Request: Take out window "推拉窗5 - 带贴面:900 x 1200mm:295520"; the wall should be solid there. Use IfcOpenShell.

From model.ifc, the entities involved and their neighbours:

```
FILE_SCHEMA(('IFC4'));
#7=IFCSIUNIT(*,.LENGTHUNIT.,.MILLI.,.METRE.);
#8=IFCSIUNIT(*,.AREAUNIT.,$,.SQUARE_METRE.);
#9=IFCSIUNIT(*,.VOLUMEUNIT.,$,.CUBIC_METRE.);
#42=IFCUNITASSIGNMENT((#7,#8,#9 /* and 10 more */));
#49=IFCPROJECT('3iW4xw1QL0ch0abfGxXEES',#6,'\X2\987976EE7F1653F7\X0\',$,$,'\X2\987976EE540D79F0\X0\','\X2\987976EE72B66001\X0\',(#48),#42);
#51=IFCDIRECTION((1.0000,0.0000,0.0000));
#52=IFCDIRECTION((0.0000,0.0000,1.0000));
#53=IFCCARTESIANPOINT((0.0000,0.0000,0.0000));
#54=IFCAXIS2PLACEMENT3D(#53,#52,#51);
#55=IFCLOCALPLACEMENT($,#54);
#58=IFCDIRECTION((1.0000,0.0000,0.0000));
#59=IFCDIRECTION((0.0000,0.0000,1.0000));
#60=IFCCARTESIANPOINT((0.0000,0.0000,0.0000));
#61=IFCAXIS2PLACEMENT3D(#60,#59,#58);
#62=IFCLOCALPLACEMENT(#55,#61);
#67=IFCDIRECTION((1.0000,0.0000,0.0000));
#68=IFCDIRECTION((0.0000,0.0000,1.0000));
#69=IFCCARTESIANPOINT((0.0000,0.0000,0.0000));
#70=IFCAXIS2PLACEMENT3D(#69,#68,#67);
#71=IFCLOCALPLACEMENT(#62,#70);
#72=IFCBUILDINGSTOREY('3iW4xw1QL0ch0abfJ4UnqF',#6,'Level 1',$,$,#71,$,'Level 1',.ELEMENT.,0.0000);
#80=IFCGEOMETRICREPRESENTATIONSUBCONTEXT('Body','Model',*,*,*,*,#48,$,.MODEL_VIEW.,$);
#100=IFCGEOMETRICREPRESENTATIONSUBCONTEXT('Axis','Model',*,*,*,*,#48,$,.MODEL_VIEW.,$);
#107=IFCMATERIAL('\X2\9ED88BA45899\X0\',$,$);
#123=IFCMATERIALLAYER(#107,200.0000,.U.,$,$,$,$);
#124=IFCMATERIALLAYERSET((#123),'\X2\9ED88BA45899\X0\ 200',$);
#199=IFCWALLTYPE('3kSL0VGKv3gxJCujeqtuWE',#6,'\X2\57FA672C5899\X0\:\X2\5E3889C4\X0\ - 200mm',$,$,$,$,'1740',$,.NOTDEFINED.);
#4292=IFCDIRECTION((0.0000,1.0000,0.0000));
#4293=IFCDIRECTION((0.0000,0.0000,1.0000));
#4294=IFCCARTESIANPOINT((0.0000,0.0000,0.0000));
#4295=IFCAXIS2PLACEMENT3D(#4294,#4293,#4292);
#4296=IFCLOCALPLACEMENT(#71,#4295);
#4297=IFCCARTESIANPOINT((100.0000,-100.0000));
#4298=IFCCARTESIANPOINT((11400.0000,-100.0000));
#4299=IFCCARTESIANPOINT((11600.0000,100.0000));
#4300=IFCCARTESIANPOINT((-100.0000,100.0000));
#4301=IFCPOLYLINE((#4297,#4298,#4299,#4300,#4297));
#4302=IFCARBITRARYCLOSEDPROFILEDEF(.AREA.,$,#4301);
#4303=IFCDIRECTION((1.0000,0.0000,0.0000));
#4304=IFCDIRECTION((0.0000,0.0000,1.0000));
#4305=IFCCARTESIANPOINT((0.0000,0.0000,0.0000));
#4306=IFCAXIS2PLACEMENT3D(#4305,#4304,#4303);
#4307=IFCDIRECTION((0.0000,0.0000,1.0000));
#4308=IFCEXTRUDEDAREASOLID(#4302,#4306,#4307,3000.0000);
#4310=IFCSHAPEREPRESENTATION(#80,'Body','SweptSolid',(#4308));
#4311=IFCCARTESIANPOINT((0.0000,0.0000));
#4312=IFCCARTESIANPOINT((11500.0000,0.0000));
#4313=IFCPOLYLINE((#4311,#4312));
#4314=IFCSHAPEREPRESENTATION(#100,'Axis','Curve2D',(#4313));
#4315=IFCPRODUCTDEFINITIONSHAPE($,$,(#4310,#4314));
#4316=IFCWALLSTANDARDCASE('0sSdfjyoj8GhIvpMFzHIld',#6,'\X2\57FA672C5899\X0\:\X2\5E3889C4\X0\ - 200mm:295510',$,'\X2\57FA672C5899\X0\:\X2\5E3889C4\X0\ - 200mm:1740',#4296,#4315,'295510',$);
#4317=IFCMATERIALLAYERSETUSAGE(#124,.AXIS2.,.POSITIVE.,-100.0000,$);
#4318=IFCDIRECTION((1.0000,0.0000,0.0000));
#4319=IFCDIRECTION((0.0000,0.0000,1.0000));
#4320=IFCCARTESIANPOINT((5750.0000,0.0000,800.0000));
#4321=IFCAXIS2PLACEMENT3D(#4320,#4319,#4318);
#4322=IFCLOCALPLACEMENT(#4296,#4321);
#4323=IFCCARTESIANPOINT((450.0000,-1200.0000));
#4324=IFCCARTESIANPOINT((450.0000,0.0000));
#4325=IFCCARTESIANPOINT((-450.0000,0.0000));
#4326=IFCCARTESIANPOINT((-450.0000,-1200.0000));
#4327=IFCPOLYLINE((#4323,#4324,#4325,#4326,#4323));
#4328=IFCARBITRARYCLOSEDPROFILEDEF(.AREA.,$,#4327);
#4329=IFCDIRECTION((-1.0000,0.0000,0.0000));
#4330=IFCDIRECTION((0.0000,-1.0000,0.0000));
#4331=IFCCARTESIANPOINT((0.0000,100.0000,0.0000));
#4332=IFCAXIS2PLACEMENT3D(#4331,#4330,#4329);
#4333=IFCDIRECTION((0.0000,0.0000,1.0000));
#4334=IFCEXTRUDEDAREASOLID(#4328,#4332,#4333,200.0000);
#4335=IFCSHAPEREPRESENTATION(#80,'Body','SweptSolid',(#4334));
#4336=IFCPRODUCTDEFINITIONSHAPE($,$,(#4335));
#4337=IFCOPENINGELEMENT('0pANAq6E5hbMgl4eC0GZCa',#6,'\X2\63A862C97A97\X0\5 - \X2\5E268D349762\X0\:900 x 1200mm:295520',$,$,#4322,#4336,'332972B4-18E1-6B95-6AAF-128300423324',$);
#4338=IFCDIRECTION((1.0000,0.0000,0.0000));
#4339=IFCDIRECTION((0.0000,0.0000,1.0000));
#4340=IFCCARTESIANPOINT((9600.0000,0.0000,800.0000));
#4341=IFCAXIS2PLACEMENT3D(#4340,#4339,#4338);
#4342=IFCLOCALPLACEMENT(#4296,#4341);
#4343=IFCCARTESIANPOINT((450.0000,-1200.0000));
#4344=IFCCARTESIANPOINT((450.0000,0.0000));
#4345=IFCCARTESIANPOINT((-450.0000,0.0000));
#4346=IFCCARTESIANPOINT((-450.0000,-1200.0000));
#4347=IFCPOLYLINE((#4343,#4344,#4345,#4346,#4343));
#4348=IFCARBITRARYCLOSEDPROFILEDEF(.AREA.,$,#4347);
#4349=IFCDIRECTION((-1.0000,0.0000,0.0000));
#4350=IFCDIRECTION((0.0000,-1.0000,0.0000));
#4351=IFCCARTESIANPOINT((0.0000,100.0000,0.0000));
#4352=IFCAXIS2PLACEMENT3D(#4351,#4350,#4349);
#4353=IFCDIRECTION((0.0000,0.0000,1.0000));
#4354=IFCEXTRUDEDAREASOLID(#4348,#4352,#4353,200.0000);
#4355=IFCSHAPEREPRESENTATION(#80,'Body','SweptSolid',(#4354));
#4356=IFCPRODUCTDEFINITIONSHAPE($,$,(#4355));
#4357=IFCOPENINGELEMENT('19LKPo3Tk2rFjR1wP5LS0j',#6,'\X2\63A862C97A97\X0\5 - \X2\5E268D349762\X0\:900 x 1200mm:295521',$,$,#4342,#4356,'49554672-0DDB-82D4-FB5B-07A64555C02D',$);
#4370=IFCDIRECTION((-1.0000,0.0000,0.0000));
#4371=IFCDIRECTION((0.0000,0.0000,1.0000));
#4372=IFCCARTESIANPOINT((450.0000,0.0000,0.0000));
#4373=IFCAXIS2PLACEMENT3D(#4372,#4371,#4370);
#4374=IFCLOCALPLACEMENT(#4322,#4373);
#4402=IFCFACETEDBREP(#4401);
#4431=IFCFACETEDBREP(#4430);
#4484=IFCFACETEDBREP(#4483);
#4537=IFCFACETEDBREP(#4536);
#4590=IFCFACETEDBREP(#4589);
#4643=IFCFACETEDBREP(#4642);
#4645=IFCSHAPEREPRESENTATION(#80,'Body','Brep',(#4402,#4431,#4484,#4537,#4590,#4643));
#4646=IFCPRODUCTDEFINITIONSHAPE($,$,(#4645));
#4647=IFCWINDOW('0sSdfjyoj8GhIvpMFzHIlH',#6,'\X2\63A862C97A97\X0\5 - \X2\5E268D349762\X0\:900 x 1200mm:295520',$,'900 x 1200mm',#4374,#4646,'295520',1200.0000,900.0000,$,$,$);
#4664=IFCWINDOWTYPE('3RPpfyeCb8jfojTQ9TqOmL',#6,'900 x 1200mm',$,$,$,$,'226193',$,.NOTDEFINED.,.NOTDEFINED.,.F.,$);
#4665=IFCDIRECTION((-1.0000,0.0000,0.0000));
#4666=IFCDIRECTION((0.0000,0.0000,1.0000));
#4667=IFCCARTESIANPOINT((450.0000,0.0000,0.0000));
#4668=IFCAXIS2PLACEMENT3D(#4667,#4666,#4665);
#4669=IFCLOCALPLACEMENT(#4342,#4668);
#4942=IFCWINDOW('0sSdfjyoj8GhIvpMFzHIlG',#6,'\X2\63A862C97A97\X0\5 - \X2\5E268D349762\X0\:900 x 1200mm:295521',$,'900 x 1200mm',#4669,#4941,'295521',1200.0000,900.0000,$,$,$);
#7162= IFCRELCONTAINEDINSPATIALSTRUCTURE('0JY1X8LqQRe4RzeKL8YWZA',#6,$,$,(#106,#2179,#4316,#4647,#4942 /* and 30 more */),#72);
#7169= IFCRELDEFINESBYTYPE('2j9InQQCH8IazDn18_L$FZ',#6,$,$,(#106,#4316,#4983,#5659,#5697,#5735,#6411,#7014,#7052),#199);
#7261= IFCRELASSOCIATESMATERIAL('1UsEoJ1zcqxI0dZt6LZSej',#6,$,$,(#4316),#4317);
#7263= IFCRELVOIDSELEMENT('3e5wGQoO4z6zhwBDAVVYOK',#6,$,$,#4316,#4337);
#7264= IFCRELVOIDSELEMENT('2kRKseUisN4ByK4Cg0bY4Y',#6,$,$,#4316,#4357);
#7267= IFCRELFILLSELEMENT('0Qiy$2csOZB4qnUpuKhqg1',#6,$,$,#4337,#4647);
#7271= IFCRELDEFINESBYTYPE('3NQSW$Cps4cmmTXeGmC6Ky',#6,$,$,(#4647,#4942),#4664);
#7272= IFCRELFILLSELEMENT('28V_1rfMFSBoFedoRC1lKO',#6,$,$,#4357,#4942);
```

```python
import ifcopenshell
import ifcopenshell.api.feature
import ifcopenshell.api.root
import ifcopenshell.geom
import ifcopenshell.util.shape

model = ifcopenshell.open("model.ifc")
settings = ifcopenshell.geom.settings()


def volume(element):
    """Net volume in cubic metres, openings subtracted."""
    shape = ifcopenshell.geom.create_shape(settings, element)
    return ifcopenshell.util.shape.get_volume(shape.geometry)


window = model.by_guid("0sSdfjyoj8GhIvpMFzHIlH")
opening = window.FillsVoids[0].RelatingOpeningElement
wall = opening.VoidsElements[0].RelatingBuildingElement
before = volume(wall)

ifcopenshell.api.root.remove_product(model, product=window)
ifcopenshell.api.feature.remove_feature(model, feature=opening)

after = volume(wall)

print(f"wall volume {before:.3f} -> {after:.3f} m3")

model.write("model_updated.ifc")
```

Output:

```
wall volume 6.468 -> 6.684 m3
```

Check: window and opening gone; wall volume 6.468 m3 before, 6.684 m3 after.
